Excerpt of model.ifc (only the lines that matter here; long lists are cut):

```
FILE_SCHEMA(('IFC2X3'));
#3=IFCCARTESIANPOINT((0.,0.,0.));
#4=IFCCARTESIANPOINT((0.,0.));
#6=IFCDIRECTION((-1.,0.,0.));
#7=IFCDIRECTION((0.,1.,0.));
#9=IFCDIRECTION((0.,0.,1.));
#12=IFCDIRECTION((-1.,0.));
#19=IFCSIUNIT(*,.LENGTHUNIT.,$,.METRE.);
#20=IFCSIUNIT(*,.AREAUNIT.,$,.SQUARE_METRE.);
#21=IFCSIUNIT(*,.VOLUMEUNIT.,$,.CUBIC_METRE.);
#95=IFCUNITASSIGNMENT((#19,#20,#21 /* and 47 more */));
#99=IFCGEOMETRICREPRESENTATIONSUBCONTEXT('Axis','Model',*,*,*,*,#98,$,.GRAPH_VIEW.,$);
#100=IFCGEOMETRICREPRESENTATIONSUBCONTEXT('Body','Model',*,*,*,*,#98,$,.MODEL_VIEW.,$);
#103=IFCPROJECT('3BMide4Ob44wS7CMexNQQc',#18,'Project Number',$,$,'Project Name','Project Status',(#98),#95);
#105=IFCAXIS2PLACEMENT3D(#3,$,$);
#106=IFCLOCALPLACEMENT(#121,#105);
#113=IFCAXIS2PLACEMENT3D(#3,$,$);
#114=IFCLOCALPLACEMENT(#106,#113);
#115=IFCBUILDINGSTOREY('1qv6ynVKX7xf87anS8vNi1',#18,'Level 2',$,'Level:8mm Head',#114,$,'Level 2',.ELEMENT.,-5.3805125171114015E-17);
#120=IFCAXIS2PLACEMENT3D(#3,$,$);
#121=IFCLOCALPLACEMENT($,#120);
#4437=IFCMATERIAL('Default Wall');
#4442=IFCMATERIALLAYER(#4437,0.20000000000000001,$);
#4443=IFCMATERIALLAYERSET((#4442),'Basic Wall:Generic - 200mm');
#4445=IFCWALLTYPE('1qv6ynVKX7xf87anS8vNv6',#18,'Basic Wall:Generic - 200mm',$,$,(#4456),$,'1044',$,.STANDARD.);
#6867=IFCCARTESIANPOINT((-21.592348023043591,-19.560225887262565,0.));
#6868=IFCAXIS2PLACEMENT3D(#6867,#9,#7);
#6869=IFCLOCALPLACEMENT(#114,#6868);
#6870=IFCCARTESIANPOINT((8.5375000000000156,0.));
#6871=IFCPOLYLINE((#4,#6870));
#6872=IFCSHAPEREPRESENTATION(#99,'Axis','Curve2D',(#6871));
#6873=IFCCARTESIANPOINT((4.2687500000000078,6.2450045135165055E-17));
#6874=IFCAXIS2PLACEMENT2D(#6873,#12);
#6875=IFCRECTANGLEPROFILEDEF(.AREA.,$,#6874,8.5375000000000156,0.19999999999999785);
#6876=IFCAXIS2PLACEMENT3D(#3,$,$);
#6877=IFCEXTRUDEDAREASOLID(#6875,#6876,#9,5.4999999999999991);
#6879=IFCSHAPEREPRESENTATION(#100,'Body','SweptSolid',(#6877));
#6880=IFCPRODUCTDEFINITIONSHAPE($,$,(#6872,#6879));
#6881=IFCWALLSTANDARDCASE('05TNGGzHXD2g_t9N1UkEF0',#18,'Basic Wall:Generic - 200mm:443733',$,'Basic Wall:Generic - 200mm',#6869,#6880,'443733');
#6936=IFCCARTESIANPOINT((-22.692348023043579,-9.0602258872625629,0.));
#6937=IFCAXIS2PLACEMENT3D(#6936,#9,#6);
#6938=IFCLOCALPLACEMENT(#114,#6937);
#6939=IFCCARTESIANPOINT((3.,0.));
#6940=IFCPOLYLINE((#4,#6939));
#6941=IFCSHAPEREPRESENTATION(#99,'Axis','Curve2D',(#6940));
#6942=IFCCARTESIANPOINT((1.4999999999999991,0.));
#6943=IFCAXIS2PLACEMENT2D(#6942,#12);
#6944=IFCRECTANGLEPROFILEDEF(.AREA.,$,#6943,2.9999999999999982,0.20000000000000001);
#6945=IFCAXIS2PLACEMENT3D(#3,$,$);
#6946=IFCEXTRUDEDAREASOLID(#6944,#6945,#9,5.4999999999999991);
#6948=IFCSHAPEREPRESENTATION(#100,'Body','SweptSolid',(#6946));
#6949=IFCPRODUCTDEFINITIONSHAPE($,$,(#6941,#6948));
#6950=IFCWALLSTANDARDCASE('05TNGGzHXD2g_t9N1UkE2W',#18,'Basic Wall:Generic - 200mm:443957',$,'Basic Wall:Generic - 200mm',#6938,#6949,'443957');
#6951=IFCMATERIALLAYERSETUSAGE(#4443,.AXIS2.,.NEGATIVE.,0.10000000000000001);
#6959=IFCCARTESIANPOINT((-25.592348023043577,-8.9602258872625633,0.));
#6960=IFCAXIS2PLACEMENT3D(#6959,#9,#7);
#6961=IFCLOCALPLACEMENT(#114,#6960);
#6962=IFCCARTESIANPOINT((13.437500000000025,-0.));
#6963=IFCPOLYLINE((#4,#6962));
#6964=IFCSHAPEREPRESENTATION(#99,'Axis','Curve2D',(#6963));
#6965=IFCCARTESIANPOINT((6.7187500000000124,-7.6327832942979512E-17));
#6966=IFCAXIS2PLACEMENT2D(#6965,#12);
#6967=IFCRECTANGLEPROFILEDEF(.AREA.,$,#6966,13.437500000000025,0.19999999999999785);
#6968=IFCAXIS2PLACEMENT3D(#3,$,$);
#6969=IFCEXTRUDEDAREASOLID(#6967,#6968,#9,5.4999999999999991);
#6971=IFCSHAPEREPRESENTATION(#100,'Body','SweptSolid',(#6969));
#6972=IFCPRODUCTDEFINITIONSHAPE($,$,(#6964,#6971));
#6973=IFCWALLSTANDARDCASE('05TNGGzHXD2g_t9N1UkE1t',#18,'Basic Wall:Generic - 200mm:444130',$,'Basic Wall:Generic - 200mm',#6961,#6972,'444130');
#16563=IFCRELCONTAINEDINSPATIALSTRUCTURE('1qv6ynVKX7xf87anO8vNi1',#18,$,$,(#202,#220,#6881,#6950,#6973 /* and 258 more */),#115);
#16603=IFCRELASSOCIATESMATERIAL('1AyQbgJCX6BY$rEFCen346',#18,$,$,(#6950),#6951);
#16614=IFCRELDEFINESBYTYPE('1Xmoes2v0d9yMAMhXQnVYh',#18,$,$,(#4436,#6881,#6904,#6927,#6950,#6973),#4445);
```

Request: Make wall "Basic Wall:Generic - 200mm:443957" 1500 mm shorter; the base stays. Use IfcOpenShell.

```python
import ifcopenshell
import ifcopenshell.geom
import ifcopenshell.util.representation
import ifcopenshell.util.shape

model = ifcopenshell.open("model.ifc")
settings = ifcopenshell.geom.settings()


def volume(element):
    """Net volume in cubic metres, openings subtracted."""
    shape = ifcopenshell.geom.create_shape(settings, element)
    return ifcopenshell.util.shape.get_volume(shape.geometry)


wall = model.by_id(6950)
before = volume(wall)

body = ifcopenshell.util.representation.get_representation(wall, "Model", "Body")
solid = body.Items[0]
old_height = solid.Depth
solid.Depth -= 1.5
after = volume(wall)

print(f"height {old_height:g} -> {solid.Depth:g}, volume {before:.3f} -> {after:.3f} m3")

model.write("model_edited.ifc")
```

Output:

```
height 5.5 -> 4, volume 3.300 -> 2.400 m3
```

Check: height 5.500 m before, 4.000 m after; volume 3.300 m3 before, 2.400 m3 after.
